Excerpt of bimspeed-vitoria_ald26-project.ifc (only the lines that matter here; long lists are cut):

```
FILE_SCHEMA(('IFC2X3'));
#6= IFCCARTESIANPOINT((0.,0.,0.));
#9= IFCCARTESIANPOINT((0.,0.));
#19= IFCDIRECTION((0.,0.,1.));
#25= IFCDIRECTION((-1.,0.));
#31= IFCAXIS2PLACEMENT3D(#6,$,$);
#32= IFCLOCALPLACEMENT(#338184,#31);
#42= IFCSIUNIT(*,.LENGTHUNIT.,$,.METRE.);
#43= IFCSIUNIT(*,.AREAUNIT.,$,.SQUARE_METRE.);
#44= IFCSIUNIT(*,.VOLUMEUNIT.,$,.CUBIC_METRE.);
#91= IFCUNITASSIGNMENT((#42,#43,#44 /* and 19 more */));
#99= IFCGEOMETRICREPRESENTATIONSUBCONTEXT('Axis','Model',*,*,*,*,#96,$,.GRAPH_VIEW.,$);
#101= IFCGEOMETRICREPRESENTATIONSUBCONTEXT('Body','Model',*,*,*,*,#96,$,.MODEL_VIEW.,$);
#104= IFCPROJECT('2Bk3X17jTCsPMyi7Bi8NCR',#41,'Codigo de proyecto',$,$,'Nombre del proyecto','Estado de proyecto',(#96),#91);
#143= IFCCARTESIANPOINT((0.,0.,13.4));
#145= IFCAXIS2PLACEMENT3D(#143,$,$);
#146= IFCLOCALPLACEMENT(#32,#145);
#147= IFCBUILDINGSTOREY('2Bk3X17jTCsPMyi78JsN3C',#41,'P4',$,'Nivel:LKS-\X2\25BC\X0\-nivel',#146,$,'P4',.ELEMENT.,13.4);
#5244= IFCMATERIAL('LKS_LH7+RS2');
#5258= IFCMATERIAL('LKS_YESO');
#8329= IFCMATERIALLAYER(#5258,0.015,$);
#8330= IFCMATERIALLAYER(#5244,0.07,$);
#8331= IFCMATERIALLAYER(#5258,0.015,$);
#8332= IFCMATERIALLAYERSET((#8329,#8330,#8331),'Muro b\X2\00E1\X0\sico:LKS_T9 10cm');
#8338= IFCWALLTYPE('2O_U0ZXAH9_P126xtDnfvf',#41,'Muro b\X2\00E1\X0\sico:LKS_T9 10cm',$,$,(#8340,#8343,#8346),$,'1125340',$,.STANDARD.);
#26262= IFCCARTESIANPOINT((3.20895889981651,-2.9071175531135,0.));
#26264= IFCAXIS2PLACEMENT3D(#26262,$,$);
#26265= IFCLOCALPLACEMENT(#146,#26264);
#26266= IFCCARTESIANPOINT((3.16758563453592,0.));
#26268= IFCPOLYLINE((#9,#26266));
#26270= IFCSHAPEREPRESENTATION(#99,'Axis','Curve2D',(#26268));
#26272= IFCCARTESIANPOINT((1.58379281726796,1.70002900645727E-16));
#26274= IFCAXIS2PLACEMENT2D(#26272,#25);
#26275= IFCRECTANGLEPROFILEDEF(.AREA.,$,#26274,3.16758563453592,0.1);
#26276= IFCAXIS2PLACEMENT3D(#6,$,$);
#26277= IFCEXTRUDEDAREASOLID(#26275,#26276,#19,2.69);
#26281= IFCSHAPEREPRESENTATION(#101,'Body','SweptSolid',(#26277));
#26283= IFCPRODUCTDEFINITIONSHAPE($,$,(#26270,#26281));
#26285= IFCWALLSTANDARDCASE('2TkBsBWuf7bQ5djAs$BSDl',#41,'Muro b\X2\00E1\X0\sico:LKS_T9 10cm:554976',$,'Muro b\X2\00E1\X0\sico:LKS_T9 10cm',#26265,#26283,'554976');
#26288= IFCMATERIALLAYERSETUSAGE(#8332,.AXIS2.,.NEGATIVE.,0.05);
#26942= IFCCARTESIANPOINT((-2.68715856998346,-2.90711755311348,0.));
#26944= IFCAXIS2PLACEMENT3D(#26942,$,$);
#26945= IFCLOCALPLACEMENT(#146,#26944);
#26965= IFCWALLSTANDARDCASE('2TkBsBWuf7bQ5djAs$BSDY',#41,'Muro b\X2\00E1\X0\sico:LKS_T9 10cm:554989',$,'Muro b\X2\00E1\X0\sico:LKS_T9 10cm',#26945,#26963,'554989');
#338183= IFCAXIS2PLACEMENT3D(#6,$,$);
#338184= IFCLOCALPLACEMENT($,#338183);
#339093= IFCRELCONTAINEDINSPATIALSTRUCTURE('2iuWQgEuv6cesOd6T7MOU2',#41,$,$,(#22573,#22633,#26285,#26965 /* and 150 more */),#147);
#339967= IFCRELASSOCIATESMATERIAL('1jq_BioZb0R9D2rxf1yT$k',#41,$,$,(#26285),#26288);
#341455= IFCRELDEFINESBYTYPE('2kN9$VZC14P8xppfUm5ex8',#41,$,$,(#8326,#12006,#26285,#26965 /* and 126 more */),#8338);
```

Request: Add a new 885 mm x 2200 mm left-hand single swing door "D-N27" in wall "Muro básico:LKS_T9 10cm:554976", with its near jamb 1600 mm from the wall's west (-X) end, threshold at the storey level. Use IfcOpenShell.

```python
import numpy as np
import ifcopenshell
import ifcopenshell.api.feature
import ifcopenshell.api.geometry
import ifcopenshell.api.root
import ifcopenshell.api.spatial
import ifcopenshell.api.type
import ifcopenshell.geom
import ifcopenshell.util.element
import ifcopenshell.util.placement
import ifcopenshell.util.representation
import ifcopenshell.util.shape
import ifcopenshell.util.unit

model = ifcopenshell.open("bimspeed-vitoria_ald26-project.ifc")
unit_scale = ifcopenshell.util.unit.calculate_unit_scale(model)
settings = ifcopenshell.geom.settings()


def volume(element):
    """Net volume in cubic metres, openings subtracted."""
    shape = ifcopenshell.geom.create_shape(settings, element)
    return ifcopenshell.util.shape.get_volume(shape.geometry)


wall = model.by_id(26285)
storey = ifcopenshell.util.element.get_container(wall, ifc_class="IfcBuildingStorey")
context = ifcopenshell.util.representation.get_context(model, "Model", "Body", "MODEL_VIEW")
before = volume(wall)

width, height, from_end, sill = 0.885, 2.2, 1.6, 0.0  # metres

# The wall runs along its own X axis, and the end named is its -X end.
wall_shape = ifcopenshell.geom.create_shape(settings, wall)
x, y, z = ifcopenshell.util.shape.get_vertices(wall_shape.geometry).T
start = x.min() + from_end
face, thickness = float(y.min()), float(y.max() - y.min())
wall_matrix = ifcopenshell.util.placement.get_local_placement(wall.ObjectPlacement)
level = ifcopenshell.util.placement.get_local_placement(storey.ObjectPlacement)[2, 3]


def in_wall(x, y):
    """Placement at x, y metres in the wall's axes, at sill height."""
    matrix = wall_matrix.copy()
    matrix[:, 3] = wall_matrix @ np.array([x / unit_scale, y / unit_scale, 0.0, 1.0])
    matrix[2, 3] = level + sill / unit_scale
    return matrix


# Opening: a box that overshoots both wall faces by 50 mm.
opening = ifcopenshell.api.root.create_entity(model, ifc_class="IfcOpeningElement")
box = ifcopenshell.api.geometry.add_wall_representation(
    model, context=context, length=width, height=height, thickness=thickness + 0.1
)
ifcopenshell.api.geometry.assign_representation(model, product=opening, representation=box)
ifcopenshell.api.geometry.edit_object_placement(model, product=opening, matrix=in_wall(start, face - 0.05), is_si=False)
ifcopenshell.api.feature.add_feature(model, feature=opening, element=wall)

door = ifcopenshell.api.root.create_entity(model, ifc_class="IfcDoor", name="D-N27")
door.OverallWidth, door.OverallHeight = width / unit_scale, height / unit_scale
body = ifcopenshell.api.geometry.add_door_representation(
    model,
    context=context,
    overall_width=door.OverallWidth,
    overall_height=door.OverallHeight,
    operation_type="SINGLE_SWING_LEFT",
    lining_properties={"LiningDepth": thickness / unit_scale, "ThresholdDepth": thickness / unit_scale},
)
ifcopenshell.api.geometry.assign_representation(model, product=door, representation=body)
ifcopenshell.api.spatial.assign_container(model, products=[door], relating_structure=storey)
fills = ifcopenshell.api.feature.add_filling(model, opening=opening, element=door)
fills.OwnerHistory = door.OwnerHistory  # required in IFC2X3

# IFC2X3 keeps the operation on the door style.
style = ifcopenshell.api.root.create_entity(model, ifc_class="IfcDoorStyle", name="D-N27")
style.OperationType, style.ConstructionType = "SINGLE_SWING_LEFT", "NOTDEFINED"
style.ParameterTakesPrecedence = style.Sizeable = False
ifcopenshell.api.type.assign_type(model, related_objects=[door], relating_type=style)

# The lining spans the wall, so the door starts at the wall face.
ifcopenshell.api.geometry.edit_object_placement(model, product=door, matrix=in_wall(start, face), is_si=False)

after = volume(wall)

print(f"wall volume {before:.3f} -> {after:.3f} m3")

model.write("bimspeed-vitoria_ald26-project-out.ifc")
```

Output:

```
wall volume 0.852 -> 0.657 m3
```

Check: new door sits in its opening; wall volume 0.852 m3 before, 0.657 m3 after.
